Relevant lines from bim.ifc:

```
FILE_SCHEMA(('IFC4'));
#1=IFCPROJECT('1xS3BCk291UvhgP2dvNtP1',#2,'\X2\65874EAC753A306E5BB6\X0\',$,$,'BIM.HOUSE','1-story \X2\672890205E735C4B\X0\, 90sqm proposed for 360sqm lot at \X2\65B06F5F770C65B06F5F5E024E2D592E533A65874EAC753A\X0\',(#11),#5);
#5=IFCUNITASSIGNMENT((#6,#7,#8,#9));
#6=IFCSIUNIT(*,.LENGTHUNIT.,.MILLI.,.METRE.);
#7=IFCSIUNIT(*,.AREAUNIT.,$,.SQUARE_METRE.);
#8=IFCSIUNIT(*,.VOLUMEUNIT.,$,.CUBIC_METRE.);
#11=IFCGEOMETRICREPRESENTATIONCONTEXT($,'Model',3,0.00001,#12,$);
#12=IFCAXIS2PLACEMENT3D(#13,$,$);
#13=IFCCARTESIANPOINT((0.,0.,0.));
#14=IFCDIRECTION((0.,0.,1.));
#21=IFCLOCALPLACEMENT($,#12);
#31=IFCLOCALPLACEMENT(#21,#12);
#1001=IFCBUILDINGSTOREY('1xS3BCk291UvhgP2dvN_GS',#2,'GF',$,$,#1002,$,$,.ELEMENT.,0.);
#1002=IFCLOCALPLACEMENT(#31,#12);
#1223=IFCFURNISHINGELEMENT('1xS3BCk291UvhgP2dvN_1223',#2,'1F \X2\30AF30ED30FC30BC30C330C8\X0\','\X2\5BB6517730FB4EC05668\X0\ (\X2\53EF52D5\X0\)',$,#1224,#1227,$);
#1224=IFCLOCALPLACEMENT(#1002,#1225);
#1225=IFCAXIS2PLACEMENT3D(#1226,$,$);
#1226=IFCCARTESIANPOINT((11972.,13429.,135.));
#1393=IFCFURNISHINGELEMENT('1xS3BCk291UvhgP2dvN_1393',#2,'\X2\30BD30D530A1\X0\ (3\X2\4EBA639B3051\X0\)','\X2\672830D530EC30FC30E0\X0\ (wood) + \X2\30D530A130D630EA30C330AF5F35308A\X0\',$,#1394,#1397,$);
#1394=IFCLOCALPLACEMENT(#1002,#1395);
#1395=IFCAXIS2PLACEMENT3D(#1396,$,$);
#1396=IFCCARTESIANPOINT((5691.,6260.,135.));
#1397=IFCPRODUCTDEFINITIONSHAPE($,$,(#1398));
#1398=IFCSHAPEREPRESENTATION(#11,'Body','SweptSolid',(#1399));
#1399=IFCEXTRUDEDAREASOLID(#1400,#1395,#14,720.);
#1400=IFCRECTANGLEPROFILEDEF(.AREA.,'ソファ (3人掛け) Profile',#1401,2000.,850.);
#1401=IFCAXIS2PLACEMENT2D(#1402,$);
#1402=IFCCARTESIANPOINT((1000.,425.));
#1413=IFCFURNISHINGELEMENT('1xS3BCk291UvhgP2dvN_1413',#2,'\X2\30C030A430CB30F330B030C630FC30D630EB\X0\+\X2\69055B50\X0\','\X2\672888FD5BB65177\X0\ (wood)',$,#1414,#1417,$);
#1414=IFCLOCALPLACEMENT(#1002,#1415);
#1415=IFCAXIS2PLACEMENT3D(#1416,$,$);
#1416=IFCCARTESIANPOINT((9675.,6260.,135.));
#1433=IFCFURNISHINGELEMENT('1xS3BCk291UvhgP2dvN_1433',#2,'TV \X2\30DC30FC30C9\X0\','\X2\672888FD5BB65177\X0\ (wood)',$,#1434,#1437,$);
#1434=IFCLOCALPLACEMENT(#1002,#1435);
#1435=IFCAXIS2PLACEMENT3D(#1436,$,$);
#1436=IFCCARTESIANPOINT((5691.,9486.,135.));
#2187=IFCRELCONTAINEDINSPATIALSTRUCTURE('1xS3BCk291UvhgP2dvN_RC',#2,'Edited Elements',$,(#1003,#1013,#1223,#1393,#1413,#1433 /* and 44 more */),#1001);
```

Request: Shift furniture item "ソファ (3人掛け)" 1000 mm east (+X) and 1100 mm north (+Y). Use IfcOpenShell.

```python
import ifcopenshell
import ifcopenshell.api.geometry
import ifcopenshell.util.placement
import ifcopenshell.util.unit

model = ifcopenshell.open("bim.ifc")
unit_scale = ifcopenshell.util.unit.calculate_unit_scale(model)

item = model.by_guid("1xS3BCk291UvhgP2dvN_1393")
matrix = ifcopenshell.util.placement.get_local_placement(item.ObjectPlacement)
matrix[0, 3] += 1 / unit_scale
matrix[1, 3] += 1.1 / unit_scale
ifcopenshell.api.geometry.edit_object_placement(model, product=item, matrix=matrix, is_si=False)

print(ifcopenshell.util.placement.get_local_placement(item.ObjectPlacement).round(3) + 0.0)

model.write("bim_edited.ifc")
```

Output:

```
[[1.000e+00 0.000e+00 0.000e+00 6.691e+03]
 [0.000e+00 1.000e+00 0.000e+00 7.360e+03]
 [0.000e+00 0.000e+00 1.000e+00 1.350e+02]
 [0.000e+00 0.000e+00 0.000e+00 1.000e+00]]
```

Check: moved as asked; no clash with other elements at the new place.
